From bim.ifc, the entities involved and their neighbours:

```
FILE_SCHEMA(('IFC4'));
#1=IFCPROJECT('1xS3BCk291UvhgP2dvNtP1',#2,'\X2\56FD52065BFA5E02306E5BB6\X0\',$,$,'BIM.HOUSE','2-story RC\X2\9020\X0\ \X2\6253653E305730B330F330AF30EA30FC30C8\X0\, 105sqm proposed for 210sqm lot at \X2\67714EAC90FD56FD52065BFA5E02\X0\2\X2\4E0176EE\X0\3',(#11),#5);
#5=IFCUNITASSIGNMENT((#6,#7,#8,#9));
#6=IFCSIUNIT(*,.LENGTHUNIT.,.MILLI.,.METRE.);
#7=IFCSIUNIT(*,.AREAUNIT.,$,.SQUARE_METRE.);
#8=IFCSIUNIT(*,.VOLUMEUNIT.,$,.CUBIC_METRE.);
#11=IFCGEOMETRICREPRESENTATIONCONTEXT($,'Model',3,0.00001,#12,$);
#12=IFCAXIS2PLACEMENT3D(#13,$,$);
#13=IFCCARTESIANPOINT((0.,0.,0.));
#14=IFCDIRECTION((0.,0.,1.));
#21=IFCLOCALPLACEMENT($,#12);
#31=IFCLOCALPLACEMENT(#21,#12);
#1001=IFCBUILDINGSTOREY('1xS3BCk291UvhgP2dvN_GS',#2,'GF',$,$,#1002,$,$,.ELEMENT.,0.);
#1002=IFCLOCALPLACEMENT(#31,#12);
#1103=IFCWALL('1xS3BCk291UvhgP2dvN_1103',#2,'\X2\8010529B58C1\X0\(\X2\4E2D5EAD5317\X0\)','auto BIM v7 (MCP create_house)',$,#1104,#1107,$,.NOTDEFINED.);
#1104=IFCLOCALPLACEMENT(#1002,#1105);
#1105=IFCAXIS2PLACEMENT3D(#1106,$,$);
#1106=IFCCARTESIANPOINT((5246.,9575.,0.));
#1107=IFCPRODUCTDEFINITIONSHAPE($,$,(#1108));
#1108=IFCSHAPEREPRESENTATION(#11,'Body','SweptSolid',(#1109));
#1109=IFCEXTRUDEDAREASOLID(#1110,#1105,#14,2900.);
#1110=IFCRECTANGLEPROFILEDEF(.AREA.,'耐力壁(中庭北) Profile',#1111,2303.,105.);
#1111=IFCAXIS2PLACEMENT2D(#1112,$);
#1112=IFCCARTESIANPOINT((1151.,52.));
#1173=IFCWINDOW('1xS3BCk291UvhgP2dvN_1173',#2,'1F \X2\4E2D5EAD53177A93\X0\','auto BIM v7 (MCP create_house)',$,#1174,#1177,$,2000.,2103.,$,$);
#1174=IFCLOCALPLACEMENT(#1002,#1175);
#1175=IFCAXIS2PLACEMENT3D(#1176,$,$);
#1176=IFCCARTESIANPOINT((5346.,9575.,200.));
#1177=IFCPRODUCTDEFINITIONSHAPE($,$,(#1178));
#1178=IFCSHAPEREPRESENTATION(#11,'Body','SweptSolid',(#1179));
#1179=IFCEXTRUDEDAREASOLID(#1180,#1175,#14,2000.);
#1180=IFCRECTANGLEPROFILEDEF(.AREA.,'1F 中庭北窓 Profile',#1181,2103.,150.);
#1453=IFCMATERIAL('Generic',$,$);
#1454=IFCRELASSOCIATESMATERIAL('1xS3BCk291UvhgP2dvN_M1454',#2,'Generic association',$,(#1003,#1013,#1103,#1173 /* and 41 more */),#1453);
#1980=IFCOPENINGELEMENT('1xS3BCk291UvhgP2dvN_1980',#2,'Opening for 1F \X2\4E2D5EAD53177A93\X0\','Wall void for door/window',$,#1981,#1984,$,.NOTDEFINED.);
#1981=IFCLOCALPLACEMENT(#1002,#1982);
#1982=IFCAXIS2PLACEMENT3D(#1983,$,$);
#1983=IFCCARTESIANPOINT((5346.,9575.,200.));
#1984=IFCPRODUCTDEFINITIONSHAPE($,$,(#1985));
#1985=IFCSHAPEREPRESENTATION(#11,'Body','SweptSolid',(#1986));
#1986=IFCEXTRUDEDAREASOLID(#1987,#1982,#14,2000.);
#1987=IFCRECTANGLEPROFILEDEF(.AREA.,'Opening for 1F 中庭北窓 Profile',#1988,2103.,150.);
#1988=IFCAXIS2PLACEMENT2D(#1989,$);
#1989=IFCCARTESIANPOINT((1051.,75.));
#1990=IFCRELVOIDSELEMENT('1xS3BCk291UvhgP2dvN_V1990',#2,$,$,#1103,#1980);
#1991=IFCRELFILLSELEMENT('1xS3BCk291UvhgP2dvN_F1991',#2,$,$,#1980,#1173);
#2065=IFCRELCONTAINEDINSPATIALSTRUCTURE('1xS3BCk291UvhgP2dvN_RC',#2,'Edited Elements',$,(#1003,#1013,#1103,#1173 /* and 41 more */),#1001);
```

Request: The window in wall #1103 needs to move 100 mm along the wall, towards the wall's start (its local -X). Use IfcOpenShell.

```python
import ifcopenshell
import ifcopenshell.api.geometry
import ifcopenshell.util.placement
import ifcopenshell.util.unit

model = ifcopenshell.open("bim.ifc")
unit_scale = ifcopenshell.util.unit.calculate_unit_scale(model)

window = model.by_guid("1xS3BCk291UvhgP2dvN_1173")
opening = window.FillsVoids[0].RelatingOpeningElement
wall = opening.VoidsElements[0].RelatingBuildingElement

wall_matrix = ifcopenshell.util.placement.get_local_placement(wall.ObjectPlacement)
shift = wall_matrix[:3, 0] * -0.1 / unit_scale
before = ifcopenshell.util.placement.get_local_placement(window.ObjectPlacement)[:3, 3].copy()

# The window is not placed relative to its opening, so move both.
for product in (opening, window):
    matrix = ifcopenshell.util.placement.get_local_placement(product.ObjectPlacement)
    matrix[:3, 3] += shift
    ifcopenshell.api.geometry.edit_object_placement(model, product=product, matrix=matrix, is_si=False)

after = ifcopenshell.util.placement.get_local_placement(window.ObjectPlacement)[:3, 3]
print("window moved by", (after - before).round(3) + 0.0)

model.write("bim_rev.ifc")
```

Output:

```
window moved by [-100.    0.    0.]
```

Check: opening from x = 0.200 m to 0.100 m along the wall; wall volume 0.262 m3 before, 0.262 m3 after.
